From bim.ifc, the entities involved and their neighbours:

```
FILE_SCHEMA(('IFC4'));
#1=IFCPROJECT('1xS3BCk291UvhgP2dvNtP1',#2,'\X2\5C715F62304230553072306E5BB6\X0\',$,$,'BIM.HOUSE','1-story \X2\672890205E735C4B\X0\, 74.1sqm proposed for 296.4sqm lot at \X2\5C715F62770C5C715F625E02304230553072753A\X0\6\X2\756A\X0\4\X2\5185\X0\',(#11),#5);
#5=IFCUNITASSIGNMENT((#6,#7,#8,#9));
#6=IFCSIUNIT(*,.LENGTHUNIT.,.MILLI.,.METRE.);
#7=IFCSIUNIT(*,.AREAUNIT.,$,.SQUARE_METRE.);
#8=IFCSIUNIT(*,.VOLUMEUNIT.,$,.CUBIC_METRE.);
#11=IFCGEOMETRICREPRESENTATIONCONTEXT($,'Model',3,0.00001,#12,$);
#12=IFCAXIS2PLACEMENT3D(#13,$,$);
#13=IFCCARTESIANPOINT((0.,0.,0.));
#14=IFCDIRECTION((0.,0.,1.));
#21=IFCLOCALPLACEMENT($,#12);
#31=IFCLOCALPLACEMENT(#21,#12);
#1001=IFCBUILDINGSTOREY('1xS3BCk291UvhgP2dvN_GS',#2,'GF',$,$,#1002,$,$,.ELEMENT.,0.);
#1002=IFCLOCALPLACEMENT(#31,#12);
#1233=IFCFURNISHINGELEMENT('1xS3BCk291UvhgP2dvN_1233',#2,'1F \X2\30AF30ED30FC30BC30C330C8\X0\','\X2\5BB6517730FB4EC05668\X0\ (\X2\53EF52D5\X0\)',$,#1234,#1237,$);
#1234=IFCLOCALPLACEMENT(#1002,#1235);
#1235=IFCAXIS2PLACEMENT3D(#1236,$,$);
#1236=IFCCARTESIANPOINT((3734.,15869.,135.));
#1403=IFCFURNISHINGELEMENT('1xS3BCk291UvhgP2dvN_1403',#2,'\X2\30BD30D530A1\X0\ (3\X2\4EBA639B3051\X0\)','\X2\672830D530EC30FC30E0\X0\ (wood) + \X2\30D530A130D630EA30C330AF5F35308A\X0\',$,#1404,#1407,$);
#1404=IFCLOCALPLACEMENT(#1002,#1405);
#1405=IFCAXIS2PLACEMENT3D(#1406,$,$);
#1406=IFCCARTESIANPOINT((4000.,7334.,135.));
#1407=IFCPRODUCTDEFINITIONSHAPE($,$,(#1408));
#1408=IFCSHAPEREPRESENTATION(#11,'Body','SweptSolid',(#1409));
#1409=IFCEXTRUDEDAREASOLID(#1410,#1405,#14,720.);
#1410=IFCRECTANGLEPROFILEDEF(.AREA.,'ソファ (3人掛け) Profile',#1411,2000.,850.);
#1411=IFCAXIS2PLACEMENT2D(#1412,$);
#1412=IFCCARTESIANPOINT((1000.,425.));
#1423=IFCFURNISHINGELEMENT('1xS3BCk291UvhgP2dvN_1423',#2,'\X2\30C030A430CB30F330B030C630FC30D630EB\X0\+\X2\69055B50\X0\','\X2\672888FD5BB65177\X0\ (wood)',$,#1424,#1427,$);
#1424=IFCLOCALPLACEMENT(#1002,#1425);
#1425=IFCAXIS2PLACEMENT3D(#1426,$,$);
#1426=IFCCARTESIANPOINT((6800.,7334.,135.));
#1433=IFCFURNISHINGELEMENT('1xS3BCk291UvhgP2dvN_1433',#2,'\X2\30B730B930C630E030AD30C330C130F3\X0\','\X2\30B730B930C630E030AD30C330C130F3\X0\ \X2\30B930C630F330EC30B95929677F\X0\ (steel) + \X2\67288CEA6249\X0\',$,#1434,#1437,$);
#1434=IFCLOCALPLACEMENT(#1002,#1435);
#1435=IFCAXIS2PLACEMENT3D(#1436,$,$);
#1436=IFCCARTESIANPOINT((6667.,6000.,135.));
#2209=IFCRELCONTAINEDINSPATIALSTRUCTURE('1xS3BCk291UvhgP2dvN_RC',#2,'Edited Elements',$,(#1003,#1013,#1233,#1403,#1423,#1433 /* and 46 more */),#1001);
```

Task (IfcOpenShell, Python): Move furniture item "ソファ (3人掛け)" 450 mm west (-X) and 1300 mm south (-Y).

```python
import ifcopenshell
import ifcopenshell.api.geometry
import ifcopenshell.util.placement

model = ifcopenshell.open("bim.ifc")

item = model.by_id(1403)
matrix = ifcopenshell.util.placement.get_local_placement(item.ObjectPlacement)
matrix[0, 3] -= 450.0
matrix[1, 3] -= 1300.0
ifcopenshell.api.geometry.edit_object_placement(model, product=item, matrix=matrix, is_si=False)

print(ifcopenshell.util.placement.get_local_placement(item.ObjectPlacement).round(3) + 0.0)

model.write("bim_rev.ifc")
```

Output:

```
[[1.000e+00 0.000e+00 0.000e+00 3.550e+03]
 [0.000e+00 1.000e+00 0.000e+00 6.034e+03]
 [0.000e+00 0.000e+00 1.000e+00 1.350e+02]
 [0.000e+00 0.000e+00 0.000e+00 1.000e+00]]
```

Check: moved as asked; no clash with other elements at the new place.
